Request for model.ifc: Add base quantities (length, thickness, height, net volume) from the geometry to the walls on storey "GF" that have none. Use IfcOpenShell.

First a look at what the model holds.

```python
import ifcopenshell
import ifcopenshell.util.element
import ifcopenshell.util.unit

model = ifcopenshell.open("model.ifc")
print(model.schema)
for unit_type in ("LENGTHUNIT", "AREAUNIT", "VOLUMEUNIT"):
    print(unit_type, ifcopenshell.util.unit.calculate_unit_scale(model, unit_type))
storey = next(s for s in model.by_type("IfcBuildingStorey") if s.Name == "GF")
walls = [e for e in ifcopenshell.util.element.get_decomposition(storey) if e.is_a("IfcWall")]
for e in sorted(walls, key=lambda e: e.id()):
    print(e.id(), e.is_a(), e.Name, list(ifcopenshell.util.element.get_psets(e, qtos_only=True)), sep=" | ")
```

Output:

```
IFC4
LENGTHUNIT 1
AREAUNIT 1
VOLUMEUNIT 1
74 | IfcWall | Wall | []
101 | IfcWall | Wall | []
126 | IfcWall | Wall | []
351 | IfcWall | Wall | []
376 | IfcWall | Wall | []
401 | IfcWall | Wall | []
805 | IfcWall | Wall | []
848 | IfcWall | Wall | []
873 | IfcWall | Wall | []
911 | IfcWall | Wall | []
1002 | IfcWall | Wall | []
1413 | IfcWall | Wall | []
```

```python
import ifcopenshell
import ifcopenshell.api.pset
import ifcopenshell.geom
import ifcopenshell.util.element
import ifcopenshell.util.shape
import ifcopenshell.util.unit

model = ifcopenshell.open("model.ifc")
unit_scale = ifcopenshell.util.unit.calculate_unit_scale(model)
volume_scale = ifcopenshell.util.unit.calculate_unit_scale(model, "VOLUMEUNIT")
settings = ifcopenshell.geom.settings()

storey = next(s for s in model.by_type("IfcBuildingStorey") if s.Name == "GF")
walls = [e for e in ifcopenshell.util.element.get_decomposition(storey) if e.is_a("IfcWall")]

for e in sorted(walls, key=lambda e: e.id()):
    if ifcopenshell.util.element.get_psets(e, qtos_only=True, should_inherit=False):
        continue
    # Geometry comes back in metres, in the element's own axes.
    shape = ifcopenshell.geom.create_shape(settings, e)
    values = {
        "Length": ifcopenshell.util.shape.get_x(shape.geometry) / unit_scale,
        "Width": ifcopenshell.util.shape.get_y(shape.geometry) / unit_scale,
        "Height": ifcopenshell.util.shape.get_z(shape.geometry) / unit_scale,
        "NetVolume": ifcopenshell.util.shape.get_volume(shape.geometry) / volume_scale,
    }
    qto = ifcopenshell.api.pset.add_qto(model, product=e, name="Qto_WallBaseQuantities")
    ifcopenshell.api.pset.edit_qto(model, qto=qto, properties=values)
    print(e.id(), {k: round(v, 3) for k, v in values.items()})

model.write("model_edited.ifc")
```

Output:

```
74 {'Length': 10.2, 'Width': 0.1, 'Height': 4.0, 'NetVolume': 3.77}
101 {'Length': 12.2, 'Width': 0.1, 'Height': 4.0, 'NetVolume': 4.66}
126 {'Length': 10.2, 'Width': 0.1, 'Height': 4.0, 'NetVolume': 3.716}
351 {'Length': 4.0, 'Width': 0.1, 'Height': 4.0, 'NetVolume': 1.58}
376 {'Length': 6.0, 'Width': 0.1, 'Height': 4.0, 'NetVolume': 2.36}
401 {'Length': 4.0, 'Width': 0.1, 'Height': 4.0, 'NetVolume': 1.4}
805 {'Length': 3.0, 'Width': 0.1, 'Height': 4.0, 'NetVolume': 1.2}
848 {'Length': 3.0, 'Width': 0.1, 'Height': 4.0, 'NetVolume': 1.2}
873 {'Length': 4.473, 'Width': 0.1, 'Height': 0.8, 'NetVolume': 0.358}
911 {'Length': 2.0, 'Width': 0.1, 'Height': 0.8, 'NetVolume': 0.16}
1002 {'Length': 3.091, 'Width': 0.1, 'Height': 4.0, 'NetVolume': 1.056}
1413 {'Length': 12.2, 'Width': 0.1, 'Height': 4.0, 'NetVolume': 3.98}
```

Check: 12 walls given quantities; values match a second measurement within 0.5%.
